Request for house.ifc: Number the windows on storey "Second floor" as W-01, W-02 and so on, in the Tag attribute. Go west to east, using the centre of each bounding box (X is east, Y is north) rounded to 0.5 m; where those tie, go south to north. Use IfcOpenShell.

First a look at what the model holds.

```python
import ifcopenshell
import ifcopenshell.util.element
import ifcopenshell.util.placement

model = ifcopenshell.open("house.ifc")
print(model.schema)
storey = next(s for s in model.by_type("IfcBuildingStorey") if s.Name == "Second floor")
windows = [e for e in ifcopenshell.util.element.get_decomposition(storey) if e.is_a("IfcWindow")]
for e in sorted(windows, key=lambda e: e.id()):
    origin = ifcopenshell.util.placement.get_local_placement(e.ObjectPlacement)[:3, 3]
    print(e.id(), e.Tag, e.Name, origin.round(2) + 0.0, sep=" | ")
```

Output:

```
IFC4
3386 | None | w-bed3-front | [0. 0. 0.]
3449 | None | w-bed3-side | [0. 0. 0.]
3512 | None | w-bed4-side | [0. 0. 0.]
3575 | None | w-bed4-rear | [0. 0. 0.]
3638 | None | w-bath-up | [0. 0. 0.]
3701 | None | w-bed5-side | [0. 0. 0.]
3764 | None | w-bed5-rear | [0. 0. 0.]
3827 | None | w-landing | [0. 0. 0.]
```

```python
import ifcopenshell
import ifcopenshell.geom
import ifcopenshell.util.element
import ifcopenshell.util.shape

model = ifcopenshell.open("house.ifc")
settings = ifcopenshell.geom.settings()
settings.set("use-world-coords", True)


def centre(element):
    shape = ifcopenshell.geom.create_shape(settings, element)
    return ifcopenshell.util.shape.get_bbox_centroid(shape.geometry)


storey = next(s for s in model.by_type("IfcBuildingStorey") if s.Name == "Second floor")
windows = [e for e in ifcopenshell.util.element.get_decomposition(storey) if e.is_a("IfcWindow")]

# Insertion points can sit at a corner or the storey origin, so sort by the geometry (in metres).
centres = {e: centre(e) for e in windows}
windows.sort(key=lambda e: (round(centres[e][0] / 0.5), centres[e][1]))

for i, e in enumerate(windows, start=1):
    number = f"W-{i:02d}"
    e.Tag = number
    print(e.id(), number)

model.write("house_edited.ifc")
```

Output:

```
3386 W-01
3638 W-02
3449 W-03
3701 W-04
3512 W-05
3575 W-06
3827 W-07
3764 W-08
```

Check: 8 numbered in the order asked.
